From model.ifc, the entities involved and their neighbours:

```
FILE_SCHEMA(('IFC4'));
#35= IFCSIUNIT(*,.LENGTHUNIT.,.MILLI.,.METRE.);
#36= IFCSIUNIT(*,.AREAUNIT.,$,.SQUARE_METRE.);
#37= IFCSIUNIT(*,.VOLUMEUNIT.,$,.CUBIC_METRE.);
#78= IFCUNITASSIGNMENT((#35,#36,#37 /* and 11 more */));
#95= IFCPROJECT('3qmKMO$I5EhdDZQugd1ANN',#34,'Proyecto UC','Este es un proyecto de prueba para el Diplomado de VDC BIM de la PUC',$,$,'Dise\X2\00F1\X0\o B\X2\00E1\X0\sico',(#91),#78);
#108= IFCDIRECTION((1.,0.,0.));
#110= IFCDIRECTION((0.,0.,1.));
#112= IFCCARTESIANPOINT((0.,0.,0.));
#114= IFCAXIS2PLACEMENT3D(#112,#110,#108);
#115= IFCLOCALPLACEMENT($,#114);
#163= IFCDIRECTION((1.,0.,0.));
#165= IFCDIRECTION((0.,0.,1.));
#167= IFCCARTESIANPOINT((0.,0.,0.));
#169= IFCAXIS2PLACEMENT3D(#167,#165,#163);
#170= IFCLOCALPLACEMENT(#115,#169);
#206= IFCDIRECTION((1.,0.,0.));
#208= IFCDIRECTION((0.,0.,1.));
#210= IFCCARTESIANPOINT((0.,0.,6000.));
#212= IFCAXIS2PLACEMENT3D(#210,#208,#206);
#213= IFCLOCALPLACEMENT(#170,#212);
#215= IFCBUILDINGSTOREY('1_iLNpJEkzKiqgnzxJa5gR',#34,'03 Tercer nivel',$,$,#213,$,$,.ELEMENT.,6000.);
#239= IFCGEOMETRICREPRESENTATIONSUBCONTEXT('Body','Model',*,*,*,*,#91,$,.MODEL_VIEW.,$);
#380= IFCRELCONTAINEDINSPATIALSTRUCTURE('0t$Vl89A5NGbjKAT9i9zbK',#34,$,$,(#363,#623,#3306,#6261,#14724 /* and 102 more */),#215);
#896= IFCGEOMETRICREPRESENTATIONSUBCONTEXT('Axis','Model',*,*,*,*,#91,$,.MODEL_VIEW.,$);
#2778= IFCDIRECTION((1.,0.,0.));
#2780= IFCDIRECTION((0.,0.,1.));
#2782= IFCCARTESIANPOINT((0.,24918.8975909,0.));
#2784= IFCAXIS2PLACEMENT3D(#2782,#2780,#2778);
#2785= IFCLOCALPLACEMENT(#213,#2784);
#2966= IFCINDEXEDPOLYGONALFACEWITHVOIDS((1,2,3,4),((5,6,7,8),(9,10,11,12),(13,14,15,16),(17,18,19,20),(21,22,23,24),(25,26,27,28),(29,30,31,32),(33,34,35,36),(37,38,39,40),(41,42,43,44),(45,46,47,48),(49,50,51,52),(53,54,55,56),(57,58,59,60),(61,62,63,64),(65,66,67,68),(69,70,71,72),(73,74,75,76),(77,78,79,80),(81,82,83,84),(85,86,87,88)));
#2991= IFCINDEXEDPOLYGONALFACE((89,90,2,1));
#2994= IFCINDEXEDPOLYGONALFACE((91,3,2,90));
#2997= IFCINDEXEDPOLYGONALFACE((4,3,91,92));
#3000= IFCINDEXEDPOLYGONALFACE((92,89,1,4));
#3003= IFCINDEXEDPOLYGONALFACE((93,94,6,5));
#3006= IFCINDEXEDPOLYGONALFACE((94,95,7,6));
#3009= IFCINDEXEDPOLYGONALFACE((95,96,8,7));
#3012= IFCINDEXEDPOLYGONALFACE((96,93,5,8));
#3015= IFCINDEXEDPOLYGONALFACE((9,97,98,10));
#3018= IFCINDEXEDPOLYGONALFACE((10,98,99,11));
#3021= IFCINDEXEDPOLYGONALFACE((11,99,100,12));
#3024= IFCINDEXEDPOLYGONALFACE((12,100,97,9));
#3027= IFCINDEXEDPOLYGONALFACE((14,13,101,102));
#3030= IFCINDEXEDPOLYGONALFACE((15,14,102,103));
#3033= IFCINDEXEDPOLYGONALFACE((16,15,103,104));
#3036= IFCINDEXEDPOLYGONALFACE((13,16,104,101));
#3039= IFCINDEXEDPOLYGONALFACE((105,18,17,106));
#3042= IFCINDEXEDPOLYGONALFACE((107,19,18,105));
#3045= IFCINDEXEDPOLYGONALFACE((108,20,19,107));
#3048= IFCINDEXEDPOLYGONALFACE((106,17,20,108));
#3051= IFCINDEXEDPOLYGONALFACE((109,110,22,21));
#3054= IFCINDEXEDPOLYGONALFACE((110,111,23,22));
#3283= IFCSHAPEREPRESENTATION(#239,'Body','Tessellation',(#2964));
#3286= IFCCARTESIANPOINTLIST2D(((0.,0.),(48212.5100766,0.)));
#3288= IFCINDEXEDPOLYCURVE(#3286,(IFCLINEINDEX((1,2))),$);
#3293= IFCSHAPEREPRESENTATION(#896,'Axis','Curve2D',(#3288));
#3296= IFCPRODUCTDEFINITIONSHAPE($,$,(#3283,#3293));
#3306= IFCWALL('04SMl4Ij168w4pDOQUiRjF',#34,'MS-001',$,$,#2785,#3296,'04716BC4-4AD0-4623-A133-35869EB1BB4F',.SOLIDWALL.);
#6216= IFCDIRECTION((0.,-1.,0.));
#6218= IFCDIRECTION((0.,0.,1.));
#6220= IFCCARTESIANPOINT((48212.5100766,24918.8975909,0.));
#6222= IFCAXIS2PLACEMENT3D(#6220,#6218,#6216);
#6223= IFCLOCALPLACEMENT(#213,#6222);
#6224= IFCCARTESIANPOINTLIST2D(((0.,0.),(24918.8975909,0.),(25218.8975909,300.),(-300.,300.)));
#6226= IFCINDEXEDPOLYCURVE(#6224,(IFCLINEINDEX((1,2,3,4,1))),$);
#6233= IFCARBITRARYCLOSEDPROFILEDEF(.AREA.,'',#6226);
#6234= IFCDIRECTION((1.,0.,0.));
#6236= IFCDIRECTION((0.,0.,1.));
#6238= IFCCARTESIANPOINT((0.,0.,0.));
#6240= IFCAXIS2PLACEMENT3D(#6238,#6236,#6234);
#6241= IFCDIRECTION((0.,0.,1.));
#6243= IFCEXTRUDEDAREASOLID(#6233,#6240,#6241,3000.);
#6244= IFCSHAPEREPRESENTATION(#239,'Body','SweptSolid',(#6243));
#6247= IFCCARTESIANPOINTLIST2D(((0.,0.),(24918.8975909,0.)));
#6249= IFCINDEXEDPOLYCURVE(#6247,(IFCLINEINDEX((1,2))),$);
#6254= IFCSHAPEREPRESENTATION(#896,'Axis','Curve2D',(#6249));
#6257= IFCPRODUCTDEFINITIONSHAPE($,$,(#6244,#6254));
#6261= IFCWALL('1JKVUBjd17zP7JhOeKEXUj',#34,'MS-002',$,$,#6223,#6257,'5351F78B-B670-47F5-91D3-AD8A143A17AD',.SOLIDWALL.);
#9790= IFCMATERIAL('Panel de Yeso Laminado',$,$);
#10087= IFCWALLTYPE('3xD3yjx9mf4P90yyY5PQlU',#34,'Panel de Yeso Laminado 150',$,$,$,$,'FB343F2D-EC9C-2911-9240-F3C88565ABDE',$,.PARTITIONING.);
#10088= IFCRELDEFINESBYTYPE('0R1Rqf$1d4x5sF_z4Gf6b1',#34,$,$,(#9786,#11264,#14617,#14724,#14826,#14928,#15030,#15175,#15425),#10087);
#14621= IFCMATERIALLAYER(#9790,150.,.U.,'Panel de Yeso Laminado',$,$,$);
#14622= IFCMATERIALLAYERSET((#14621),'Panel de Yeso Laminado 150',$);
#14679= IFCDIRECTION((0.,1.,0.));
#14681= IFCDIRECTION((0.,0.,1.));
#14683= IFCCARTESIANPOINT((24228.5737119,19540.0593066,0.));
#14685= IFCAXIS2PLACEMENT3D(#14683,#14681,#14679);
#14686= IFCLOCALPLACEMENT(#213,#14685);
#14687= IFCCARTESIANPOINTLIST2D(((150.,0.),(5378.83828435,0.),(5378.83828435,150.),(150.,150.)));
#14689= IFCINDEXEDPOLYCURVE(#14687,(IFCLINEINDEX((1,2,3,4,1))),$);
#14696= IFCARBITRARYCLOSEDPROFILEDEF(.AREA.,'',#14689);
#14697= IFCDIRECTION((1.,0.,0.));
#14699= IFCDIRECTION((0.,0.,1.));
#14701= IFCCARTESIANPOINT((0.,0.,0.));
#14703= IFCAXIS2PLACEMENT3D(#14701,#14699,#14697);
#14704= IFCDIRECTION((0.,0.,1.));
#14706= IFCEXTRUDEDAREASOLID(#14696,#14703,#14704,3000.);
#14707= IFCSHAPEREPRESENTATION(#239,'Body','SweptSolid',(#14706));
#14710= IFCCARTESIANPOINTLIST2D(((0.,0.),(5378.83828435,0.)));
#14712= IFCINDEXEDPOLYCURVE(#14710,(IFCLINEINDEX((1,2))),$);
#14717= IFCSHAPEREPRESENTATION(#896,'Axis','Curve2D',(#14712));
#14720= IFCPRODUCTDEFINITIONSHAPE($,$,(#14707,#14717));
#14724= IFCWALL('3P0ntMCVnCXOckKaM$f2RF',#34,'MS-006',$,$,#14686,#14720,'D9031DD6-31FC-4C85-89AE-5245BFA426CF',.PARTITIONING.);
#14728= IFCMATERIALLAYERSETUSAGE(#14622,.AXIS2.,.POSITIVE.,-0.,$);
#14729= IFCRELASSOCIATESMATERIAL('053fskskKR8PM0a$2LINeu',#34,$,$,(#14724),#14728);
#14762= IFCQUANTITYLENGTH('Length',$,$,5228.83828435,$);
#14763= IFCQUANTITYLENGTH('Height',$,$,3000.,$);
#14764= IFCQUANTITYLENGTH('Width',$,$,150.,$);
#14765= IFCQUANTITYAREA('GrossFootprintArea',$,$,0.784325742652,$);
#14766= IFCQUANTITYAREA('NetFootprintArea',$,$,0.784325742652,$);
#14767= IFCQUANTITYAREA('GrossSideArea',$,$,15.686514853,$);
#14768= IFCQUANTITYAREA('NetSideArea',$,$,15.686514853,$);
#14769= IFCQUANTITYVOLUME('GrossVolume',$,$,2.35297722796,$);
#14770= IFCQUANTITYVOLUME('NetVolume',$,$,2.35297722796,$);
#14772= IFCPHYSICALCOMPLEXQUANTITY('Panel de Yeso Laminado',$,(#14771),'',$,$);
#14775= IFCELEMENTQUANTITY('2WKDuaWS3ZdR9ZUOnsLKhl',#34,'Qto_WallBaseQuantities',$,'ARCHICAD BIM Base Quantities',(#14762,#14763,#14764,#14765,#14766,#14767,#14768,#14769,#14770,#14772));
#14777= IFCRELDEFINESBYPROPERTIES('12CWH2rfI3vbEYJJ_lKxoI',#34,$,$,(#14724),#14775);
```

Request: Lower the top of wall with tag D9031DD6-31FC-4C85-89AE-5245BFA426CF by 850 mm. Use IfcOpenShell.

```python
import ifcopenshell
import ifcopenshell.api.pset
import ifcopenshell.geom
import ifcopenshell.util.element
import ifcopenshell.util.representation
import ifcopenshell.util.shape
import ifcopenshell.util.unit

model = ifcopenshell.open("model.ifc")
unit_scale = ifcopenshell.util.unit.calculate_unit_scale(model)
area_scale = ifcopenshell.util.unit.calculate_unit_scale(model, "AREAUNIT")
volume_scale = ifcopenshell.util.unit.calculate_unit_scale(model, "VOLUMEUNIT")
settings = ifcopenshell.geom.settings()


def volume(element):
    """Net volume in cubic metres, openings subtracted."""
    shape = ifcopenshell.geom.create_shape(settings, element)
    return ifcopenshell.util.shape.get_volume(shape.geometry)


wall = model.by_guid("3P0ntMCVnCXOckKaM$f2RF")
before = volume(wall)

body = ifcopenshell.util.representation.get_representation(wall, "Model", "Body")
solid = body.Items[0]
old_height = solid.Depth
solid.Depth -= 0.85 / unit_scale
after = volume(wall)
thickness = 0.15  # wall thickness in metres

# Update the stored height, areas and volumes.
qto = model.by_id(ifcopenshell.util.element.get_pset(wall, "Qto_WallBaseQuantities", should_inherit=False)["id"])
ifcopenshell.api.pset.edit_qto(model, qto=qto, properties={
    "Height": solid.Depth,
    "GrossSideArea": ifcopenshell.util.element.get_pset(wall, "Qto_WallBaseQuantities", "GrossSideArea") * solid.Depth / old_height,
    "NetSideArea": after / thickness / area_scale,
    "GrossVolume": ifcopenshell.util.element.get_pset(wall, "Qto_WallBaseQuantities", "GrossVolume") * solid.Depth / old_height,
    "NetVolume": after / volume_scale,
})

print(f"height {old_height:g} -> {solid.Depth:g}, volume {before:.3f} -> {after:.3f} m3")

model.write("model_rev.ifc")
```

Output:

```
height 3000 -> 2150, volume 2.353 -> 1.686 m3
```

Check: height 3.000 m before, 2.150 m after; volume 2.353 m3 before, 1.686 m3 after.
